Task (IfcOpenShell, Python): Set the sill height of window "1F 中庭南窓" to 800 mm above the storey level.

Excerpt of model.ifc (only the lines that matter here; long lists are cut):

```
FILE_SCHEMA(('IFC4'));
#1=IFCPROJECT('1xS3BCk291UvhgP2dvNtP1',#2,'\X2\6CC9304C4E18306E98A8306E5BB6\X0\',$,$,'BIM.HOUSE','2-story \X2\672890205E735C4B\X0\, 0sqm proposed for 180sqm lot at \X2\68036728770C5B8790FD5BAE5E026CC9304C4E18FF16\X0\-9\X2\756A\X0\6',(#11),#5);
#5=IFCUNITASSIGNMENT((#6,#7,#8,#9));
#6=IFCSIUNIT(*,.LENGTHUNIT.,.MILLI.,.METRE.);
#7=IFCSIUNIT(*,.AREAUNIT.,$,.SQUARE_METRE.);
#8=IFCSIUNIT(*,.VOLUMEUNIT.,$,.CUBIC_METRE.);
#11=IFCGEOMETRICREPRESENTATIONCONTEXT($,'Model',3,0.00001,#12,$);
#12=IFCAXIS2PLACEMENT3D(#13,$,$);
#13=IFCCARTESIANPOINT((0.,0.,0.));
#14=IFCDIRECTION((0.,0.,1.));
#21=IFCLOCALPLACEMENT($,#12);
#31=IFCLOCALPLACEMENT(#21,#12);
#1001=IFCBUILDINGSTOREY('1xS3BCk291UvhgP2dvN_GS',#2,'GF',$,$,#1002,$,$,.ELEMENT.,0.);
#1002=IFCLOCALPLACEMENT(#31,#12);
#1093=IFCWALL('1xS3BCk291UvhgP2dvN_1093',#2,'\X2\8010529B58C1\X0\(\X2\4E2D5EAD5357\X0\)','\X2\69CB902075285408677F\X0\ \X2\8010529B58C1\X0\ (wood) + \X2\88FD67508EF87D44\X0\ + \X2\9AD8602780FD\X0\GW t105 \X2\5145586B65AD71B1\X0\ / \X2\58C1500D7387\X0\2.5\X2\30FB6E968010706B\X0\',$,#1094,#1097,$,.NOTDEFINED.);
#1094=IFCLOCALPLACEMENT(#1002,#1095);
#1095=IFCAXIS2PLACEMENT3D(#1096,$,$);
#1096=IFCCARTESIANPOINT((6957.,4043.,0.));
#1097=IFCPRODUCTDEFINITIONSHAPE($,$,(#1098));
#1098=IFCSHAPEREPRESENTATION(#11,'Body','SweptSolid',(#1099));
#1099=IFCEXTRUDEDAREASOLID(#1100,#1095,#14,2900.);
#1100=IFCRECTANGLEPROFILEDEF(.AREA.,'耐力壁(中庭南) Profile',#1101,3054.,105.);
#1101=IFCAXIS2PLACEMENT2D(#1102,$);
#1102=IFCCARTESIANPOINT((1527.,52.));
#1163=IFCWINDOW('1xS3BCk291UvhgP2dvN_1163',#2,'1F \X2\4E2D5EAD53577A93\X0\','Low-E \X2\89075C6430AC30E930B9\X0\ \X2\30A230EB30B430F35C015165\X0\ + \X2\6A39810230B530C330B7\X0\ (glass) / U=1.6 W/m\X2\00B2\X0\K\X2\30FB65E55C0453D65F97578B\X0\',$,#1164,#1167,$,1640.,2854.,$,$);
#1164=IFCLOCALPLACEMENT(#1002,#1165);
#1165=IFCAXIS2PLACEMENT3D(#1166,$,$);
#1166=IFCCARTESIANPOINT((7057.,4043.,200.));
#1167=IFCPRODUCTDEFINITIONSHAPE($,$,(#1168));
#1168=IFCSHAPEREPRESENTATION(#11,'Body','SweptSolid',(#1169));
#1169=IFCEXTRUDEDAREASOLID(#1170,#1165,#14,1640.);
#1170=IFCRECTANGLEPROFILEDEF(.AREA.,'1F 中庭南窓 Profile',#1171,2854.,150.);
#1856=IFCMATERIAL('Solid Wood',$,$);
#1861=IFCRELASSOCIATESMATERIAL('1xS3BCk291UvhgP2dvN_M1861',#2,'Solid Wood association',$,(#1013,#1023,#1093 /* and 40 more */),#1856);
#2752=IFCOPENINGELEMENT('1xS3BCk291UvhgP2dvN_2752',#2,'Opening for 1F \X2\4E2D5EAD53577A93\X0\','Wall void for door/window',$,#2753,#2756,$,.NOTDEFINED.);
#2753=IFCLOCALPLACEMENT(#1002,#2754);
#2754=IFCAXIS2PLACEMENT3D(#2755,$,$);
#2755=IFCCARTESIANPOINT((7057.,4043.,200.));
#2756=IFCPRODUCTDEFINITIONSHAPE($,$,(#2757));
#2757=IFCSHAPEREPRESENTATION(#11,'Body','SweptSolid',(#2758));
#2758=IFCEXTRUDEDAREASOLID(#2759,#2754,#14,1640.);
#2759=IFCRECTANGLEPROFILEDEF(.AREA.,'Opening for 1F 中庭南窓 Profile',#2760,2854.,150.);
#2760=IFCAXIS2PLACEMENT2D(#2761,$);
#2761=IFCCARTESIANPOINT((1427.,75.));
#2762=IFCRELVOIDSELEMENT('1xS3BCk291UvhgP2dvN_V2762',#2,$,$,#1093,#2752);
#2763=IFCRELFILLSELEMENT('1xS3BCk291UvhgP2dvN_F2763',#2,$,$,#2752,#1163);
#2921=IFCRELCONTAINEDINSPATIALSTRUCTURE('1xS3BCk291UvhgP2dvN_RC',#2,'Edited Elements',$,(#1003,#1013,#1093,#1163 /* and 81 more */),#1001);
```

```python
import numpy as np
import ifcopenshell
import ifcopenshell.api.geometry
import ifcopenshell.geom
import ifcopenshell.util.element
import ifcopenshell.util.placement
import ifcopenshell.util.shape
import ifcopenshell.util.unit

model = ifcopenshell.open("model.ifc")
unit_scale = ifcopenshell.util.unit.calculate_unit_scale(model)

window = model.by_guid("1xS3BCk291UvhgP2dvN_1163")
opening = window.FillsVoids[0].RelatingOpeningElement
storey = ifcopenshell.util.element.get_container(window, ifc_class="IfcBuildingStorey")
level = ifcopenshell.util.placement.get_local_placement(storey.ObjectPlacement)[2, 3]

# The opening's origin need not be at the sill, so measure its lowest point.
shape = ifcopenshell.geom.create_shape(ifcopenshell.geom.settings(), opening)
bottom = ifcopenshell.util.shape.get_shape_bottom_elevation(shape, shape.geometry) / unit_scale
dz = level + 800.0 - bottom

shift = np.array([0.0, 0.0, dz])
# The window is not placed relative to its opening, so move both.
for product in (opening, window):
    matrix = ifcopenshell.util.placement.get_local_placement(product.ObjectPlacement)
    matrix[:3, 3] += shift
    ifcopenshell.api.geometry.edit_object_placement(model, product=product, matrix=matrix, is_si=False)

print(f"moved by {dz * unit_scale:+.3f} m")

model.write("model_updated.ifc")
```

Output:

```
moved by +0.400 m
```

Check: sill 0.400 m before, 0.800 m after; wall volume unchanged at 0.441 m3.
